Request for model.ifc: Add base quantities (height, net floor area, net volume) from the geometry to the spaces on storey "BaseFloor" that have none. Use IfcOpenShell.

First a look at what the model holds.

```python
import ifcopenshell
import ifcopenshell.util.element
import ifcopenshell.util.unit

model = ifcopenshell.open("model.ifc")
print(model.schema)
for unit_type in ("LENGTHUNIT", "AREAUNIT", "VOLUMEUNIT"):
    print(unit_type, ifcopenshell.util.unit.calculate_unit_scale(model, unit_type))
storey = next(s for s in model.by_type("IfcBuildingStorey") if s.Name == "BaseFloor")
spaces = [e for e in ifcopenshell.util.element.get_decomposition(storey) if e.is_a("IfcSpace")]
for e in sorted(spaces, key=lambda e: e.id()):
    print(e.id(), e.is_a(), e.Name, list(ifcopenshell.util.element.get_psets(e, qtos_only=True)), sep=" | ")
```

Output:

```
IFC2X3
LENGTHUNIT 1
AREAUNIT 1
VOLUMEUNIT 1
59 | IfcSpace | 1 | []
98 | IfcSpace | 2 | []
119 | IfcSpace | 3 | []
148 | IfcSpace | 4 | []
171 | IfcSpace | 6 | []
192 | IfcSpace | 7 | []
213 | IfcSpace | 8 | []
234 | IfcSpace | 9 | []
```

```python
import ifcopenshell
import ifcopenshell.api.pset
import ifcopenshell.geom
import ifcopenshell.util.element
import ifcopenshell.util.shape
import ifcopenshell.util.unit

model = ifcopenshell.open("model.ifc")
unit_scale = ifcopenshell.util.unit.calculate_unit_scale(model)
area_scale = ifcopenshell.util.unit.calculate_unit_scale(model, "AREAUNIT")
volume_scale = ifcopenshell.util.unit.calculate_unit_scale(model, "VOLUMEUNIT")
settings = ifcopenshell.geom.settings()

storey = next(s for s in model.by_type("IfcBuildingStorey") if s.Name == "BaseFloor")
spaces = [e for e in ifcopenshell.util.element.get_decomposition(storey) if e.is_a("IfcSpace")]

for e in sorted(spaces, key=lambda e: e.id()):
    if ifcopenshell.util.element.get_psets(e, qtos_only=True, should_inherit=False):
        continue
    # Geometry comes back in metres, in the element's own axes.
    shape = ifcopenshell.geom.create_shape(settings, e)
    values = {
        "Height": ifcopenshell.util.shape.get_z(shape.geometry) / unit_scale,
        "NetFloorArea": ifcopenshell.util.shape.get_footprint_area(shape.geometry) / area_scale,
        "NetVolume": ifcopenshell.util.shape.get_volume(shape.geometry) / volume_scale,
    }
    qto = ifcopenshell.api.pset.add_qto(model, product=e, name="BaseQuantities")
    ifcopenshell.api.pset.edit_qto(model, qto=qto, properties=values)
    print(e.id(), {k: round(v, 3) for k, v in values.items()})

model.write("model-out.ifc")
```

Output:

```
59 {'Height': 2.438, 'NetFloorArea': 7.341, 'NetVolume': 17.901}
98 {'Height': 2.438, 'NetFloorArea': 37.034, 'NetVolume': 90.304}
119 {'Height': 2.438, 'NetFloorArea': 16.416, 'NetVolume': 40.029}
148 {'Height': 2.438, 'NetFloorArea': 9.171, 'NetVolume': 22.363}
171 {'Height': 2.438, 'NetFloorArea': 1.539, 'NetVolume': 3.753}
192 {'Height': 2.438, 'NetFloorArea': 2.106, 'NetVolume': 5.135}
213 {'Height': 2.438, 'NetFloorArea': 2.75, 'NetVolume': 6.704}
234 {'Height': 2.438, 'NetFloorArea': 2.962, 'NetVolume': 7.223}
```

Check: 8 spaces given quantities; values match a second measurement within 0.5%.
